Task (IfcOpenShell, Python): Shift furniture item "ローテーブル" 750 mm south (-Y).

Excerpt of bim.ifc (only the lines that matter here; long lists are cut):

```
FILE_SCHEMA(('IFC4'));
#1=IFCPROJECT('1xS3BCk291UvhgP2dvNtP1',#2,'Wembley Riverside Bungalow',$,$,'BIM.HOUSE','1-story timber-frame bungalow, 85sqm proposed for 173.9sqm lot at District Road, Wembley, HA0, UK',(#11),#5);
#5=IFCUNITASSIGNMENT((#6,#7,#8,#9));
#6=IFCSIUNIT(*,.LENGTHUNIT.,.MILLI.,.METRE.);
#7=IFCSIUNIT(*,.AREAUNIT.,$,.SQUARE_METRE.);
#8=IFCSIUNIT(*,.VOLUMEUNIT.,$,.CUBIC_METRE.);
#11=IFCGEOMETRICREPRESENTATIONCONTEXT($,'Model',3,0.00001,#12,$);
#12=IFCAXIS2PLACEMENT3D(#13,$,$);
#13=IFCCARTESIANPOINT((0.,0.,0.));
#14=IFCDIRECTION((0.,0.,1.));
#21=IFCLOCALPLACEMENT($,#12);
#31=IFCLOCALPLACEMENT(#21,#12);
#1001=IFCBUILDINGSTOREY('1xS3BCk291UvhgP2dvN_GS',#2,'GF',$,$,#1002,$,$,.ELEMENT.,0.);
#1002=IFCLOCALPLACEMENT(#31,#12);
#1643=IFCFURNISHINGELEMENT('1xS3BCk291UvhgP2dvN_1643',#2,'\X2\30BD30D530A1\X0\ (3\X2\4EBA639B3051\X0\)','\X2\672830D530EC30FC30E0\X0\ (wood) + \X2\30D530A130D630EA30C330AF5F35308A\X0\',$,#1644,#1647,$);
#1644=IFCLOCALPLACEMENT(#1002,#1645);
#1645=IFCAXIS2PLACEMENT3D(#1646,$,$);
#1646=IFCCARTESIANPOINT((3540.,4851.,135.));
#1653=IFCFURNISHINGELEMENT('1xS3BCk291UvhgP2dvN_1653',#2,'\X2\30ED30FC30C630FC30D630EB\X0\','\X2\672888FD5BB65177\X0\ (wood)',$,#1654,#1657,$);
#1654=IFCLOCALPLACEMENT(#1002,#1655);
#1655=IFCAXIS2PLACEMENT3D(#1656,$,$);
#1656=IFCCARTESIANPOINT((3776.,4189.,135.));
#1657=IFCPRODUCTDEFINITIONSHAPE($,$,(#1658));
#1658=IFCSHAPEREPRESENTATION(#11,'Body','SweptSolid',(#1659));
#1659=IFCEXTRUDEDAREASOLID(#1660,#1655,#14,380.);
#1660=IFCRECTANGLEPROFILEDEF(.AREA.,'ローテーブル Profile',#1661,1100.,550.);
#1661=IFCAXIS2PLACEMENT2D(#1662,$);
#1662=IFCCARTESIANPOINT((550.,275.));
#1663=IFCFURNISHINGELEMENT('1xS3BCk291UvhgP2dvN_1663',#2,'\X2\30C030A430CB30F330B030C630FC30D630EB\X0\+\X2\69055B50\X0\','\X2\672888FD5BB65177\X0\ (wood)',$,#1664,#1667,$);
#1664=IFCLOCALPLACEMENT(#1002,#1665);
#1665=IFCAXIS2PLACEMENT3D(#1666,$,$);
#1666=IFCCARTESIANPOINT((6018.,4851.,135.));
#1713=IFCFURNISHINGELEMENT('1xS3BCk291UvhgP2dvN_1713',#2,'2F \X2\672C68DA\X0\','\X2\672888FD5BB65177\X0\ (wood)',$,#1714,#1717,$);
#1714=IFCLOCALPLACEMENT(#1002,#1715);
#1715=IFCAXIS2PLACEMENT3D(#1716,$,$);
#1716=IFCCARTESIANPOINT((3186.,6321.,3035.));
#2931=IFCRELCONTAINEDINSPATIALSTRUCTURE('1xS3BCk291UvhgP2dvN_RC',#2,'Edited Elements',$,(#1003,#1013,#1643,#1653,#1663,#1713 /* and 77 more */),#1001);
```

```python
import ifcopenshell
import ifcopenshell.api.geometry
import ifcopenshell.util.placement
import ifcopenshell.util.unit

model = ifcopenshell.open("bim.ifc")
unit_scale = ifcopenshell.util.unit.calculate_unit_scale(model)

item = model.by_guid("1xS3BCk291UvhgP2dvN_1653")
matrix = ifcopenshell.util.placement.get_local_placement(item.ObjectPlacement)
matrix[1, 3] -= 0.75 / unit_scale
ifcopenshell.api.geometry.edit_object_placement(model, product=item, matrix=matrix, is_si=False)

print(ifcopenshell.util.placement.get_local_placement(item.ObjectPlacement).round(3) + 0.0)

model.write("bim_rev.ifc")
```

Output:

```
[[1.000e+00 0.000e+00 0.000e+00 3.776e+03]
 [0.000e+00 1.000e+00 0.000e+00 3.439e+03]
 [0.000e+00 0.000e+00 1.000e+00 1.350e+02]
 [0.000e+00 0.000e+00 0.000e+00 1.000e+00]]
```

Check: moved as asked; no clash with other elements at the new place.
